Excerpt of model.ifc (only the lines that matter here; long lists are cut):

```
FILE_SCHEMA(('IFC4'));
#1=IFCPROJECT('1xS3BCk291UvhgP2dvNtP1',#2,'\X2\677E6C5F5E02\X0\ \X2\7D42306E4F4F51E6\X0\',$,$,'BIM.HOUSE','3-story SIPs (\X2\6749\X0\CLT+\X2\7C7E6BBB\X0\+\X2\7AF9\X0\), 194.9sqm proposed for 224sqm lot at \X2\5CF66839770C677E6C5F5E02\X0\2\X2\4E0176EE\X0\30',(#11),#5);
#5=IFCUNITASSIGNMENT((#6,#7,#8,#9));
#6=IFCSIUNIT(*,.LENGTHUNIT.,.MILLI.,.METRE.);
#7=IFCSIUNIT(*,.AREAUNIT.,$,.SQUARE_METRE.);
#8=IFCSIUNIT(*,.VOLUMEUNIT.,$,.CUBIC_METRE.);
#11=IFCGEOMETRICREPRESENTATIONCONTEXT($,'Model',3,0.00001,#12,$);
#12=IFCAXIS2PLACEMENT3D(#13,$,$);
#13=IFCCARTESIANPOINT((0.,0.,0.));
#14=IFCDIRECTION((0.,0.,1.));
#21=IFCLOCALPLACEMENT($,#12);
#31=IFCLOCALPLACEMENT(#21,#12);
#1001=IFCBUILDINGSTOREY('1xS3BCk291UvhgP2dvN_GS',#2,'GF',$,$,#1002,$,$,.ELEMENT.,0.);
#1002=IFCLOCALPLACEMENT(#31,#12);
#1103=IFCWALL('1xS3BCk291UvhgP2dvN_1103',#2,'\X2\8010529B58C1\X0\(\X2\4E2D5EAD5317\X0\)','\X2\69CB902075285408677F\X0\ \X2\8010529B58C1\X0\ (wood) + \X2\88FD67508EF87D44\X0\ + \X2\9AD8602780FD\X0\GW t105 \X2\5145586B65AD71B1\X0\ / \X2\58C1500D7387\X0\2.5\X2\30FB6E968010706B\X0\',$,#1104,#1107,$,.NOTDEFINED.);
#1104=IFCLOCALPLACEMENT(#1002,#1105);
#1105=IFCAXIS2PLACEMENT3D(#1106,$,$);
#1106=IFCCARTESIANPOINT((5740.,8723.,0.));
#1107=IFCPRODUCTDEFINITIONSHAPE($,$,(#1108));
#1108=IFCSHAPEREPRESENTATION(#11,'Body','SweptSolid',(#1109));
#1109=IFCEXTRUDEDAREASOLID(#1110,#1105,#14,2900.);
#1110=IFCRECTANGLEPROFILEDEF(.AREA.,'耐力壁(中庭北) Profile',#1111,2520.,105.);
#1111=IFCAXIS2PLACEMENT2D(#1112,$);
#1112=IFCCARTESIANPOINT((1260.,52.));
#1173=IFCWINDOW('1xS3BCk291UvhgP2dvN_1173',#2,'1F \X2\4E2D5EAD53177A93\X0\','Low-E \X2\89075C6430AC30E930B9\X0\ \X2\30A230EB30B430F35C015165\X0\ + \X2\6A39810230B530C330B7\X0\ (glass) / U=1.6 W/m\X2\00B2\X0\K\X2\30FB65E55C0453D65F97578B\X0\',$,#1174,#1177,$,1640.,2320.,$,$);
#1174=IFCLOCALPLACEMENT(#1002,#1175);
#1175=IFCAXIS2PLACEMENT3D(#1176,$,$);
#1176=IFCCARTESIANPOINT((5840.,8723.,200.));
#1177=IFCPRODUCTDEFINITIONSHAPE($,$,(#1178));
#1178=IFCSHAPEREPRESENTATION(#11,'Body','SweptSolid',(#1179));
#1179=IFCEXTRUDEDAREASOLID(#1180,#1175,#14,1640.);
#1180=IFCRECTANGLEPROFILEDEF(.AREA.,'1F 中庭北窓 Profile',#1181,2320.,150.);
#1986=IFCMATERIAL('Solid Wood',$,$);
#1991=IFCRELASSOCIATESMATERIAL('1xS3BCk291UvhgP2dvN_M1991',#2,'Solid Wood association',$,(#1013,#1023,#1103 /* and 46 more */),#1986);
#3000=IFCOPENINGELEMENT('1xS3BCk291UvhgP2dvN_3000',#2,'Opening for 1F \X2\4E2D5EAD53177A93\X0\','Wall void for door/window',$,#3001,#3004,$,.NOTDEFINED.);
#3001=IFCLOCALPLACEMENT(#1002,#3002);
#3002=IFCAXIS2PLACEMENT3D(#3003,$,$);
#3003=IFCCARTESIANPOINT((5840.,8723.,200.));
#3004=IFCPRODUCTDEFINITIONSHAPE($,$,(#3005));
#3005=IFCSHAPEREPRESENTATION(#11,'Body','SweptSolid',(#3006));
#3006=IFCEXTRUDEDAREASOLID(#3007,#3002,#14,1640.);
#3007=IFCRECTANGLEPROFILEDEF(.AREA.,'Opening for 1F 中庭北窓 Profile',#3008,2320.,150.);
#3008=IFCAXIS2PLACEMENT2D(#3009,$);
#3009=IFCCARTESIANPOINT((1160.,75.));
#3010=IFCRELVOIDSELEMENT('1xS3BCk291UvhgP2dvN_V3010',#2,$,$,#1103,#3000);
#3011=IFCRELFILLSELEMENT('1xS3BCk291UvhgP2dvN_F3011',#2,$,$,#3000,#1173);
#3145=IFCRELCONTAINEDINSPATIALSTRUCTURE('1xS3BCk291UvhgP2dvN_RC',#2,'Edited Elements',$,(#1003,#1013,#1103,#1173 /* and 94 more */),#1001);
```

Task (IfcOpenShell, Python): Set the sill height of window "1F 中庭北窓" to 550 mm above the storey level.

```python
import numpy as np
import ifcopenshell
import ifcopenshell.api.geometry
import ifcopenshell.geom
import ifcopenshell.util.element
import ifcopenshell.util.placement
import ifcopenshell.util.shape
import ifcopenshell.util.unit

model = ifcopenshell.open("model.ifc")
unit_scale = ifcopenshell.util.unit.calculate_unit_scale(model)

window = model.by_guid("1xS3BCk291UvhgP2dvN_1173")
opening = window.FillsVoids[0].RelatingOpeningElement
storey = ifcopenshell.util.element.get_container(window, ifc_class="IfcBuildingStorey")
level = ifcopenshell.util.placement.get_local_placement(storey.ObjectPlacement)[2, 3]

# The opening's origin need not be at the sill, so measure its lowest point.
shape = ifcopenshell.geom.create_shape(ifcopenshell.geom.settings(), opening)
bottom = ifcopenshell.util.shape.get_shape_bottom_elevation(shape, shape.geometry) / unit_scale
dz = level + 0.55 / unit_scale - bottom

shift = np.array([0.0, 0.0, dz])
# The window is not placed relative to its opening, so move both.
for product in (opening, window):
    matrix = ifcopenshell.util.placement.get_local_placement(product.ObjectPlacement)
    matrix[:3, 3] += shift
    ifcopenshell.api.geometry.edit_object_placement(model, product=product, matrix=matrix, is_si=False)

print(f"moved by {dz * unit_scale:+.3f} m")

model.write("model_updated.ifc")
```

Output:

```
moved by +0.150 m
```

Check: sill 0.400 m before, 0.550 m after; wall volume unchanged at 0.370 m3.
